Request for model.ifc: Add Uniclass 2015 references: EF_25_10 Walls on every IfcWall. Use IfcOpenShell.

First a look at what the model holds.

```python
import ifcopenshell

model = ifcopenshell.open("model.ifc")
print(model.schema)
print("classifications:", [c.Name for c in model.by_type("IfcClassification")])
for ifc_class in ("IfcDoor", "IfcRoof", "IfcStair", "IfcWall", "IfcWindow"):
    print(ifc_class, len(model.by_type(ifc_class)))
```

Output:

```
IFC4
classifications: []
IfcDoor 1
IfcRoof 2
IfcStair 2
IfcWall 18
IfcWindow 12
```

```python
import ifcopenshell
import ifcopenshell.api.classification

model = ifcopenshell.open("model.ifc")

system = ifcopenshell.api.classification.add_classification(model, classification="Uniclass 2015")

codes = {
    "IfcWall": ("EF_25_10", "Walls"),
}
for ifc_class, (code, name) in codes.items():
    products = model.by_type(ifc_class)
    ifcopenshell.api.classification.add_reference(
        model, products=products, classification=system, identification=code, name=name
    )
    print(code, len(products))

model.write("model_updated.ifc")
```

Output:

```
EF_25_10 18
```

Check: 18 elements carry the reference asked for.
